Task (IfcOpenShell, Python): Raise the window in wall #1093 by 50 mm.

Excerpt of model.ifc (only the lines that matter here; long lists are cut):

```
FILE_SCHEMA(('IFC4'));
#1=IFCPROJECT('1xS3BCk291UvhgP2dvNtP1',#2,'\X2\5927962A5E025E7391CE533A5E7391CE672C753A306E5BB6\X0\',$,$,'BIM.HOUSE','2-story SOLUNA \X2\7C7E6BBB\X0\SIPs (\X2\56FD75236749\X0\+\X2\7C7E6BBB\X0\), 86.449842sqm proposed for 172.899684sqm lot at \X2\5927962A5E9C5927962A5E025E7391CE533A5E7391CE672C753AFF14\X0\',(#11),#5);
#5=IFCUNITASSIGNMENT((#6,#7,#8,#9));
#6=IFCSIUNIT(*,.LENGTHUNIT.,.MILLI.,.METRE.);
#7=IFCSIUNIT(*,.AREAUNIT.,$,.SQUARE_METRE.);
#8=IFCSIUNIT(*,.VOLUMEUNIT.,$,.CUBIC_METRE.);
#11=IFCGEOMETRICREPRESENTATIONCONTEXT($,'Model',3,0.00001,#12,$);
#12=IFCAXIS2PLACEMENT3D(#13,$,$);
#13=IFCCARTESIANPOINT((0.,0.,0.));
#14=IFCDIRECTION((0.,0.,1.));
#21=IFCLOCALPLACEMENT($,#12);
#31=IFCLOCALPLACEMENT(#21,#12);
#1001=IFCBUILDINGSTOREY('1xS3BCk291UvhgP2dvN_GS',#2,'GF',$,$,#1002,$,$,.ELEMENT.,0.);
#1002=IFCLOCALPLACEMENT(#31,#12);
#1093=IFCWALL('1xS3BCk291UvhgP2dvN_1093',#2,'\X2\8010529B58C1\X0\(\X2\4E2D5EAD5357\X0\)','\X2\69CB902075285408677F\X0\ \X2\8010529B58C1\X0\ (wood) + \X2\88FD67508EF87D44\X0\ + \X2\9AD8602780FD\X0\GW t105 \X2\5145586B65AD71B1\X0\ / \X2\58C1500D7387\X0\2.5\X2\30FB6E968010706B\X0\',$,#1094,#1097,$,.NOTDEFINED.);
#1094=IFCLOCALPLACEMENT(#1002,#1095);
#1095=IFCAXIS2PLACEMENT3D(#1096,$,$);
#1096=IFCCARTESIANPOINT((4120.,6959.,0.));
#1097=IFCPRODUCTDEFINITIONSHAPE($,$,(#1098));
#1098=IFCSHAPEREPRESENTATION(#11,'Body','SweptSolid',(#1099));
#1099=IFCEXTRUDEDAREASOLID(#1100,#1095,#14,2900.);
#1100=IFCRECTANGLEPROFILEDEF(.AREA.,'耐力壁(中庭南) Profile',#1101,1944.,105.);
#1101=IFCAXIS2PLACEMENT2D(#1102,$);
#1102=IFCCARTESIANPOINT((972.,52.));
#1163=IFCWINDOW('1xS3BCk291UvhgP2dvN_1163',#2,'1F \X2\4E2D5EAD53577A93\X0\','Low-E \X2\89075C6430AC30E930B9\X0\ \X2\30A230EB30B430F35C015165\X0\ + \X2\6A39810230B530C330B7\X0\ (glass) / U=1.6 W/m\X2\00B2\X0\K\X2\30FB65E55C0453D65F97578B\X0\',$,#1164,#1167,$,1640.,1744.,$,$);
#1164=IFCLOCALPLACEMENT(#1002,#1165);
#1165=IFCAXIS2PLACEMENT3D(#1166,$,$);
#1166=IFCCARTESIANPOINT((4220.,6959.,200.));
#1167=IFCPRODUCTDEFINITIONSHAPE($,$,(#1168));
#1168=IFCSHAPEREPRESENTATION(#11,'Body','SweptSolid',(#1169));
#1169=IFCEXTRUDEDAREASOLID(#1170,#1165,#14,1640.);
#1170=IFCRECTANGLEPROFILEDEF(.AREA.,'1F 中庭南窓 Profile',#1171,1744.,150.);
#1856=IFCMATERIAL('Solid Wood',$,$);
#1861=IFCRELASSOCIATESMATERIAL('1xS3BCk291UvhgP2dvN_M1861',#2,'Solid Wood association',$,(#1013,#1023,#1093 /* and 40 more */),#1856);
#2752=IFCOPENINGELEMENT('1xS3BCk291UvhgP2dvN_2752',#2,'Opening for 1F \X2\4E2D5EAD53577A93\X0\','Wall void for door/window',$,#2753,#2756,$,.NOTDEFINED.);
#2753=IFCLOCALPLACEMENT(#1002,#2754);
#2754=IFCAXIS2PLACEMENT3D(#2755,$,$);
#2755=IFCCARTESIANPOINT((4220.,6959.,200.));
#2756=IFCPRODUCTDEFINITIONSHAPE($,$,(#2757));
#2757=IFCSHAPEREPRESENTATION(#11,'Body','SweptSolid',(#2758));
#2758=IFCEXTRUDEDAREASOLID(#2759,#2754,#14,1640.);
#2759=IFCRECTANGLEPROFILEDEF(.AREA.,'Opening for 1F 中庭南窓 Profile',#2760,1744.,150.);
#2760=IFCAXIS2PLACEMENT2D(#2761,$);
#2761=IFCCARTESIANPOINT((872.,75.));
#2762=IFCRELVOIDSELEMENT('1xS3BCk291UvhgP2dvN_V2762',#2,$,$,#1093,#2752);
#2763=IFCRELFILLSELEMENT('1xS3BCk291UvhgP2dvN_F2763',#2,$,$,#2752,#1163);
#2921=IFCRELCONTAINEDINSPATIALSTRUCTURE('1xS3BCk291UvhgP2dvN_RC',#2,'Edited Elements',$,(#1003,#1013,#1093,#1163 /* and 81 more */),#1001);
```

```python
import numpy as np
import ifcopenshell
import ifcopenshell.api.geometry
import ifcopenshell.util.placement
import ifcopenshell.util.unit

model = ifcopenshell.open("model.ifc")
unit_scale = ifcopenshell.util.unit.calculate_unit_scale(model)

window = model.by_guid("1xS3BCk291UvhgP2dvN_1163")
opening = window.FillsVoids[0].RelatingOpeningElement
dz = 0.05 / unit_scale

shift = np.array([0.0, 0.0, dz])
# The window is not placed relative to its opening, so move both.
for product in (opening, window):
    matrix = ifcopenshell.util.placement.get_local_placement(product.ObjectPlacement)
    matrix[:3, 3] += shift
    ifcopenshell.api.geometry.edit_object_placement(model, product=product, matrix=matrix, is_si=False)

print(f"moved by {dz * unit_scale:+.3f} m")

model.write("model_edited.ifc")
```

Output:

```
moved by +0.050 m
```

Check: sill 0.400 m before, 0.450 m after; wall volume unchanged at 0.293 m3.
